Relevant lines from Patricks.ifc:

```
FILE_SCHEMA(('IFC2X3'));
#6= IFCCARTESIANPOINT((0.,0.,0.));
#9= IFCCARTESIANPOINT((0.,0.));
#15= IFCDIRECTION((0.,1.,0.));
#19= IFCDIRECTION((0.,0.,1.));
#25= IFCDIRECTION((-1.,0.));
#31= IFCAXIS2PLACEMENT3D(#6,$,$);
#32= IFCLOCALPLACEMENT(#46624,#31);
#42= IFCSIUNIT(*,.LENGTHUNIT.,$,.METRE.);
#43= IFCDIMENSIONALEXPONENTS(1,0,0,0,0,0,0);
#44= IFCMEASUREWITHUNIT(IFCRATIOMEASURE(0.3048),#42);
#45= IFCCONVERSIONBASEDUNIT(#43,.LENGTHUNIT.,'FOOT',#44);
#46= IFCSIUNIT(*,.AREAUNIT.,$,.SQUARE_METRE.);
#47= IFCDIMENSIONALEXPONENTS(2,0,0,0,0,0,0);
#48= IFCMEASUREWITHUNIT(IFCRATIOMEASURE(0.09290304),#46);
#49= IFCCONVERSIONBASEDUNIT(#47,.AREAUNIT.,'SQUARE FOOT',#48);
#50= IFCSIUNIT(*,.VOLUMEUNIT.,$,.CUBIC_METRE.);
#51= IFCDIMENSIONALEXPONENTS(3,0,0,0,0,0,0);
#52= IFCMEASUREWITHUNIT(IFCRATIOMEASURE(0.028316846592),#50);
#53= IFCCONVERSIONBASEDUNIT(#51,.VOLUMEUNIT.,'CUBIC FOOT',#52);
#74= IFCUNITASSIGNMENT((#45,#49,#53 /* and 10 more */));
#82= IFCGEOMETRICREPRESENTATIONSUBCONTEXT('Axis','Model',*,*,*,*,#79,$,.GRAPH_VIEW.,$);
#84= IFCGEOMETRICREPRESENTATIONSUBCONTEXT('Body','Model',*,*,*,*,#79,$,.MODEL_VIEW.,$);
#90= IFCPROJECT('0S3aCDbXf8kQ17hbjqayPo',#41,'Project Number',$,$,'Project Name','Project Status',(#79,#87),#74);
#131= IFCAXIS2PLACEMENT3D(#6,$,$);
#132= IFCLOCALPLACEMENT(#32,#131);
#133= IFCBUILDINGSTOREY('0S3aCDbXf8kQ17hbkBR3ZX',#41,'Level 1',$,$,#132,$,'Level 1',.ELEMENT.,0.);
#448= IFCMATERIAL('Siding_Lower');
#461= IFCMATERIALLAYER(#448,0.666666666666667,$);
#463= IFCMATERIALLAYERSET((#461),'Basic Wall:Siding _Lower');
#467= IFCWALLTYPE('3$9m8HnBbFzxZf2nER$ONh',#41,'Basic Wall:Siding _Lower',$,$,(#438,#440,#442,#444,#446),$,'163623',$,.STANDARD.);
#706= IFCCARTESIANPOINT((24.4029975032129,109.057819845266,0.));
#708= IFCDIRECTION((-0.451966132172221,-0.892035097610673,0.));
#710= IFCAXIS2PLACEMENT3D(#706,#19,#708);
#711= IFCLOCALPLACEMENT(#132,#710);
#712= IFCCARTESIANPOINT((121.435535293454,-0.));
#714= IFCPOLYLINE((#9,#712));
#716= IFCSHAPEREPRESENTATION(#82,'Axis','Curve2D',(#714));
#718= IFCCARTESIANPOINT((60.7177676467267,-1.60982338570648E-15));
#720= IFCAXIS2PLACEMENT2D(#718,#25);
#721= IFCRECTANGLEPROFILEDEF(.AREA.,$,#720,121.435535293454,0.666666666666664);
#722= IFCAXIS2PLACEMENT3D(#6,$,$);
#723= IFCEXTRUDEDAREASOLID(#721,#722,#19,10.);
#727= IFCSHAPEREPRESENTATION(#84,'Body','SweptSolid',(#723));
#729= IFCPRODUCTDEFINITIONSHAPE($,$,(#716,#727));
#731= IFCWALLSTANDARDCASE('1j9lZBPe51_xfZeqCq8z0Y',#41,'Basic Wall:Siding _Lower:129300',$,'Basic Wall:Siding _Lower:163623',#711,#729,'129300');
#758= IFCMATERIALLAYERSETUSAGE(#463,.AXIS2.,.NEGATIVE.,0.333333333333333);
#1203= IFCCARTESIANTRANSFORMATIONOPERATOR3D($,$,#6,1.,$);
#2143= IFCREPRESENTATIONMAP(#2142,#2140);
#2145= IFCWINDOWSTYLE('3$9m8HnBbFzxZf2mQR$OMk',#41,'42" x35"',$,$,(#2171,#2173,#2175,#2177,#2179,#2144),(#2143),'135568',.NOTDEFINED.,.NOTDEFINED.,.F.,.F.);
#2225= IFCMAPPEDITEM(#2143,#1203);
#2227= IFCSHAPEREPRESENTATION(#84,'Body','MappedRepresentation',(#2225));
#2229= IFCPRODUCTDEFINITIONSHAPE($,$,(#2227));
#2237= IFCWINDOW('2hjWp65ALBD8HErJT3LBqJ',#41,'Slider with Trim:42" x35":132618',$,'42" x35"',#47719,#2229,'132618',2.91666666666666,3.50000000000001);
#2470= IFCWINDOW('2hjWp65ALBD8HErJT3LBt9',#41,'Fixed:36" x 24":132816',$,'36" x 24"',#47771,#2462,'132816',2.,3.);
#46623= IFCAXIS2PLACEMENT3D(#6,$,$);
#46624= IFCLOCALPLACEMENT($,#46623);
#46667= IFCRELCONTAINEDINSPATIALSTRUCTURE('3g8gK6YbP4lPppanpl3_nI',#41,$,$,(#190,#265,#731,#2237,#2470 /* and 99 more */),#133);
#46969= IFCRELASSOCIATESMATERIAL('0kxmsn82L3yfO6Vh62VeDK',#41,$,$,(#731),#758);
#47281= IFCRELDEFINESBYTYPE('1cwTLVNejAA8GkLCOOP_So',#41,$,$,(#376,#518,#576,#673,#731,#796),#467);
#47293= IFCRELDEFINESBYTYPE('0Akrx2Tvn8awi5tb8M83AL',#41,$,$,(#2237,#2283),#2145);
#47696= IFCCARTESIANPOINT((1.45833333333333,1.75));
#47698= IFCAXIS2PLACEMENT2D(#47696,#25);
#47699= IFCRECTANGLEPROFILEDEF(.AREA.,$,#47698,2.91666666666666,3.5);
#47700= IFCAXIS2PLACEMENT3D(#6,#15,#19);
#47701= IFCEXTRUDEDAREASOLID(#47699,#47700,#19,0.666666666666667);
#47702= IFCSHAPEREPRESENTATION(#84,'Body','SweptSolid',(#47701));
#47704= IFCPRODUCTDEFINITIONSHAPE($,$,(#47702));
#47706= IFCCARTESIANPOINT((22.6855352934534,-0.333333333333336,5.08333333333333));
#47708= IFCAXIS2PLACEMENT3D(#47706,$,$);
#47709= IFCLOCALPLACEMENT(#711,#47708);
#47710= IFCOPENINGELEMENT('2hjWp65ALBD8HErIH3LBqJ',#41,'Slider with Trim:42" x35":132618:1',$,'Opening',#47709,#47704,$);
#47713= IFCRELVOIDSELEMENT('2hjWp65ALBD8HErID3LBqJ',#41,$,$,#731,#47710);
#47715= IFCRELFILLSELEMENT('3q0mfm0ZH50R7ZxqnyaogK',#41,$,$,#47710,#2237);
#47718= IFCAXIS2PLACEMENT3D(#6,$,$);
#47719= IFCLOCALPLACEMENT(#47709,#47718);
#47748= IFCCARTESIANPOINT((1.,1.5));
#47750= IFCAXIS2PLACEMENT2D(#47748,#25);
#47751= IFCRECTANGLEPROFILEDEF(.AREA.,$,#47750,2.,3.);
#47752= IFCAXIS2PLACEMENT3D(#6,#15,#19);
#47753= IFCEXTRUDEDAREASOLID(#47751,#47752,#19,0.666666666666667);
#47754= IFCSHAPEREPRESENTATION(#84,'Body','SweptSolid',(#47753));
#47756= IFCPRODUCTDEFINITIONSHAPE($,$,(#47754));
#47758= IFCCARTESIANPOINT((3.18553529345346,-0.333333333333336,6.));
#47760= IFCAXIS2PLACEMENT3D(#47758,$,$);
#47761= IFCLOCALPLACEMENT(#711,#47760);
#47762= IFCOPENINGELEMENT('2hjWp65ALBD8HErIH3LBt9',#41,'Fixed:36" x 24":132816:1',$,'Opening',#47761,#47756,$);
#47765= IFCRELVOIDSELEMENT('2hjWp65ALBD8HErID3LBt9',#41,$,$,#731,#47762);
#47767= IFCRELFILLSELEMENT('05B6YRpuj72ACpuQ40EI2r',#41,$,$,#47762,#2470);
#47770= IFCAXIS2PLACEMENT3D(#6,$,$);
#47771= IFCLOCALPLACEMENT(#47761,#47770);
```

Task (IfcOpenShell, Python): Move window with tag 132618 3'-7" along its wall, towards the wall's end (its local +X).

```python
import ifcopenshell
import ifcopenshell.api.geometry
import ifcopenshell.util.placement
import ifcopenshell.util.unit

model = ifcopenshell.open("Patricks.ifc")
unit_scale = ifcopenshell.util.unit.calculate_unit_scale(model)

window = model.by_id(2237)
opening = window.FillsVoids[0].RelatingOpeningElement
wall = opening.VoidsElements[0].RelatingBuildingElement

wall_matrix = ifcopenshell.util.placement.get_local_placement(wall.ObjectPlacement)
shift = wall_matrix[:3, 0] * 43 * 0.0254 / unit_scale
before = ifcopenshell.util.placement.get_local_placement(window.ObjectPlacement)[:3, 3].copy()

# The window is placed relative to its opening, so it follows when the opening moves.
matrix = ifcopenshell.util.placement.get_local_placement(opening.ObjectPlacement)
matrix[:3, 3] += shift
ifcopenshell.api.geometry.edit_object_placement(
    model, product=opening, matrix=matrix, is_si=False, should_transform_children=True
)

after = ifcopenshell.util.placement.get_local_placement(window.ObjectPlacement)[:3, 3]
print("window moved by", (after - before).round(3) + 0.0)

model.write("Patricks_rev.ifc")
```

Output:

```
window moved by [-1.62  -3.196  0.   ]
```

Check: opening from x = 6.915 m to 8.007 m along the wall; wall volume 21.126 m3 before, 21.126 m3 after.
